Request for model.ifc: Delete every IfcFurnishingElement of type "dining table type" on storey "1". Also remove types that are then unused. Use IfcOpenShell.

First a look at what the model holds.

```python
import ifcopenshell
import ifcopenshell.util.element

model = ifcopenshell.open("model.ifc")
print(model.schema)
storey = next(s for s in model.by_type("IfcBuildingStorey") if s.Name == "1")
furniture = [e for e in ifcopenshell.util.element.get_decomposition(storey) if e.is_a("IfcFurnishingElement")]
seen = {}
for e in furniture:
    element_type = ifcopenshell.util.element.get_type(e)
    name = element_type.Name if element_type not in (None, e) else None
    seen[name] = seen.get(name, 0) + 1
for name, count in sorted(seen.items(), key=str):
    print(count, "x", name)
```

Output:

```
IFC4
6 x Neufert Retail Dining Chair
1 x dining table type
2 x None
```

```python
import ifcopenshell
import ifcopenshell.api.root
import ifcopenshell.util.element

model = ifcopenshell.open("model.ifc")

storey = next(s for s in model.by_type("IfcBuildingStorey") if s.Name == "1")
furniture = [e for e in ifcopenshell.util.element.get_decomposition(storey) if e.is_a("IfcFurnishingElement")]
targets = [e for e in furniture if (t := ifcopenshell.util.element.get_type(e)) not in (None, e) and t.Name == "dining table type"]
types = {ifcopenshell.util.element.get_type(e) for e in targets} - {None, *targets}

for e in targets:
    ifcopenshell.api.root.remove_product(model, product=e)
print(len(targets), "removed")

unused = [t for t in types if not ifcopenshell.util.element.get_types(t)]
for t in unused:
    ifcopenshell.api.root.remove_product(model, product=t)
print(len(unused), "unused types removed")

model.write("model-out.ifc")
```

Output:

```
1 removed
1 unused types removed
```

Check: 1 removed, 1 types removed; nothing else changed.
